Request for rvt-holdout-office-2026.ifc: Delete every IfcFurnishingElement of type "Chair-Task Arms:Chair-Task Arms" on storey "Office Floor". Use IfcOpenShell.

First a look at what the model holds.

```python
import ifcopenshell
import ifcopenshell.util.element

model = ifcopenshell.open("rvt-holdout-office-2026.ifc")
print(model.schema)
storey = next(s for s in model.by_type("IfcBuildingStorey") if s.Name == "Office Floor")
furniture = [e for e in ifcopenshell.util.element.get_decomposition(storey) if e.is_a("IfcFurnishingElement")]
seen = {}
for e in furniture:
    element_type = ifcopenshell.util.element.get_type(e)
    name = element_type.Name if element_type not in (None, e) else None
    seen[name] = seen.get(name, 0) + 1
for name, count in sorted(seen.items(), key=str):
    print(count, "x", name)
```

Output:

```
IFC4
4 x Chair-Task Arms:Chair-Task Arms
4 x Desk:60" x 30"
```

```python
import ifcopenshell
import ifcopenshell.api.root
import ifcopenshell.util.element

model = ifcopenshell.open("rvt-holdout-office-2026.ifc")

storey = next(s for s in model.by_type("IfcBuildingStorey") if s.Name == "Office Floor")
furniture = [e for e in ifcopenshell.util.element.get_decomposition(storey) if e.is_a("IfcFurnishingElement")]
targets = [e for e in furniture if (t := ifcopenshell.util.element.get_type(e)) not in (None, e) and t.Name == "Chair-Task Arms:Chair-Task Arms"]

for e in targets:
    ifcopenshell.api.root.remove_product(model, product=e)
print(len(targets), "removed")

model.write("rvt-holdout-office-2026_rev.ifc")
```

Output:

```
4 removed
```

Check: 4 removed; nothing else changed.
